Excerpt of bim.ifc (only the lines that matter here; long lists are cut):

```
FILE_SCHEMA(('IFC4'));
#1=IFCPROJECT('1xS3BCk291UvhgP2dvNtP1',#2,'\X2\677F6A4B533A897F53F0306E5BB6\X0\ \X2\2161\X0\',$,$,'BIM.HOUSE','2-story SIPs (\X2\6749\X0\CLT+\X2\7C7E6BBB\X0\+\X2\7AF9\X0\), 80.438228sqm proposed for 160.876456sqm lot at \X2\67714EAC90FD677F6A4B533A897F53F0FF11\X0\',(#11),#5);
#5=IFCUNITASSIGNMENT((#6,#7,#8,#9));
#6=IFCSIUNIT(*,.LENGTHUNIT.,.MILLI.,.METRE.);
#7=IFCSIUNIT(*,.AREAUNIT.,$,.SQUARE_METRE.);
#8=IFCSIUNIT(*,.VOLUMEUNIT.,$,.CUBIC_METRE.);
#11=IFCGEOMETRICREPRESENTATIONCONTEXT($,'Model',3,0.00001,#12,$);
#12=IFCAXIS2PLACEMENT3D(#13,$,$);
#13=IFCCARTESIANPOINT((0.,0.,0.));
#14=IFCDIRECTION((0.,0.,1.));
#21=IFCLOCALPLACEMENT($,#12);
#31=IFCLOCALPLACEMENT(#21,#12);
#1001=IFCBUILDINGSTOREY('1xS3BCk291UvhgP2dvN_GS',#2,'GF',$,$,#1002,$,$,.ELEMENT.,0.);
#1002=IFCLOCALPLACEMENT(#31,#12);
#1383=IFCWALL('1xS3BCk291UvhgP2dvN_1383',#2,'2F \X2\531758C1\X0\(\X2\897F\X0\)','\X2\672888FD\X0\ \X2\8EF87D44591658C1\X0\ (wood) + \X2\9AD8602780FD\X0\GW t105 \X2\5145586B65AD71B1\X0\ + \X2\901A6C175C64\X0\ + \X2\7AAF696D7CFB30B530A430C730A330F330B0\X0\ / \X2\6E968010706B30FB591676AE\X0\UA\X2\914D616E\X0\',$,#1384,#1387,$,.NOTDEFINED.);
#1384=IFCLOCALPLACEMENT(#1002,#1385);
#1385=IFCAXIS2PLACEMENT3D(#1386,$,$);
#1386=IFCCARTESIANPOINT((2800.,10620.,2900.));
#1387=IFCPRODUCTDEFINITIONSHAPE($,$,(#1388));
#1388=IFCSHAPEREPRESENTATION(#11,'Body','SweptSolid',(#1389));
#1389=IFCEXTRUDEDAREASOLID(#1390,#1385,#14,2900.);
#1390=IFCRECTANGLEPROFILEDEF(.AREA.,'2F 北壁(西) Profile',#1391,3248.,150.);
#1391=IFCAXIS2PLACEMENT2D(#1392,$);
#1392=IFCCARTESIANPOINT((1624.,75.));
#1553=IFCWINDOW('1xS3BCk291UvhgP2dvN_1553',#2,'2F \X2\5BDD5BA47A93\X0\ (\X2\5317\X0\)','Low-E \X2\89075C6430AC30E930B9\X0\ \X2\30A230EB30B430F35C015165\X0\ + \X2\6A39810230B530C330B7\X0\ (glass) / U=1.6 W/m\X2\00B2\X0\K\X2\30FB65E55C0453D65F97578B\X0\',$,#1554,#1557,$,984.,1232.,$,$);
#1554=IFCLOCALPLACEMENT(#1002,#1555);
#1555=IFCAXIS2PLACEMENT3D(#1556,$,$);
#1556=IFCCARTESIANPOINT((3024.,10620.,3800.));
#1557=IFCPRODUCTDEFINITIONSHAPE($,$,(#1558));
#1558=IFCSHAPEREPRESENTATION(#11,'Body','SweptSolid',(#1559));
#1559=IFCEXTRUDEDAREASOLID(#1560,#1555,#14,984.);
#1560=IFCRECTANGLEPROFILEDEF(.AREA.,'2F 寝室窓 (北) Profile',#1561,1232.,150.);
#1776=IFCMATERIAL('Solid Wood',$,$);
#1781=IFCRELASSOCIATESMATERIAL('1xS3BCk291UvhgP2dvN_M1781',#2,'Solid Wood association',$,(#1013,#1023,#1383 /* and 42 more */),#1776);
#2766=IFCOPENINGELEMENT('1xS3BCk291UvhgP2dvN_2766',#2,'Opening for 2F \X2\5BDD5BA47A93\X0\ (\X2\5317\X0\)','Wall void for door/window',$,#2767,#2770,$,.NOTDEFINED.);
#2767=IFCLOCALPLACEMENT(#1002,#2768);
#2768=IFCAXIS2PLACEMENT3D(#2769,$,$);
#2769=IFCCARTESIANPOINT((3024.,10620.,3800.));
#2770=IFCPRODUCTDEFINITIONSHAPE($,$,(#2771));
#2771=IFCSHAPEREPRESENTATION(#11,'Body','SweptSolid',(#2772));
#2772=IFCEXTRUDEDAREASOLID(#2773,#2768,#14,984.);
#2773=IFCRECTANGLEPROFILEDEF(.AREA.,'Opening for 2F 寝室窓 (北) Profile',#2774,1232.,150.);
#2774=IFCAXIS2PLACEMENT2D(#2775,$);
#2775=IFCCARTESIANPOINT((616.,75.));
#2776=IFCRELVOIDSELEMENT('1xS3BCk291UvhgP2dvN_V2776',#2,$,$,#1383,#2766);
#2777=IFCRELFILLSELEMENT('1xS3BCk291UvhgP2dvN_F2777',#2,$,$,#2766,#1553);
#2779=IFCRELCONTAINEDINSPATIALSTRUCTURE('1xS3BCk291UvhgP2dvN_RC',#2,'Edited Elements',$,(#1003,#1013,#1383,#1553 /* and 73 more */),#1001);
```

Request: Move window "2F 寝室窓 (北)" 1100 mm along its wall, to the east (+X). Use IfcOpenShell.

```python
import ifcopenshell
import ifcopenshell.api.geometry
import ifcopenshell.util.placement
import ifcopenshell.util.unit

model = ifcopenshell.open("bim.ifc")
unit_scale = ifcopenshell.util.unit.calculate_unit_scale(model)

window = model.by_guid("1xS3BCk291UvhgP2dvN_1553")
opening = window.FillsVoids[0].RelatingOpeningElement
wall = opening.VoidsElements[0].RelatingBuildingElement

wall_matrix = ifcopenshell.util.placement.get_local_placement(wall.ObjectPlacement)
shift = wall_matrix[:3, 0] * 1.1 / unit_scale
before = ifcopenshell.util.placement.get_local_placement(window.ObjectPlacement)[:3, 3].copy()

# The window is not placed relative to its opening, so move both.
for product in (opening, window):
    matrix = ifcopenshell.util.placement.get_local_placement(product.ObjectPlacement)
    matrix[:3, 3] += shift
    ifcopenshell.api.geometry.edit_object_placement(model, product=product, matrix=matrix, is_si=False)

after = ifcopenshell.util.placement.get_local_placement(window.ObjectPlacement)[:3, 3]
print("window moved by", (after - before).round(3) + 0.0)

model.write("bim_rev.ifc")
```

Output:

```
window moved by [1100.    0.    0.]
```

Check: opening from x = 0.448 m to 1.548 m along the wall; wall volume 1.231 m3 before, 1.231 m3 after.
